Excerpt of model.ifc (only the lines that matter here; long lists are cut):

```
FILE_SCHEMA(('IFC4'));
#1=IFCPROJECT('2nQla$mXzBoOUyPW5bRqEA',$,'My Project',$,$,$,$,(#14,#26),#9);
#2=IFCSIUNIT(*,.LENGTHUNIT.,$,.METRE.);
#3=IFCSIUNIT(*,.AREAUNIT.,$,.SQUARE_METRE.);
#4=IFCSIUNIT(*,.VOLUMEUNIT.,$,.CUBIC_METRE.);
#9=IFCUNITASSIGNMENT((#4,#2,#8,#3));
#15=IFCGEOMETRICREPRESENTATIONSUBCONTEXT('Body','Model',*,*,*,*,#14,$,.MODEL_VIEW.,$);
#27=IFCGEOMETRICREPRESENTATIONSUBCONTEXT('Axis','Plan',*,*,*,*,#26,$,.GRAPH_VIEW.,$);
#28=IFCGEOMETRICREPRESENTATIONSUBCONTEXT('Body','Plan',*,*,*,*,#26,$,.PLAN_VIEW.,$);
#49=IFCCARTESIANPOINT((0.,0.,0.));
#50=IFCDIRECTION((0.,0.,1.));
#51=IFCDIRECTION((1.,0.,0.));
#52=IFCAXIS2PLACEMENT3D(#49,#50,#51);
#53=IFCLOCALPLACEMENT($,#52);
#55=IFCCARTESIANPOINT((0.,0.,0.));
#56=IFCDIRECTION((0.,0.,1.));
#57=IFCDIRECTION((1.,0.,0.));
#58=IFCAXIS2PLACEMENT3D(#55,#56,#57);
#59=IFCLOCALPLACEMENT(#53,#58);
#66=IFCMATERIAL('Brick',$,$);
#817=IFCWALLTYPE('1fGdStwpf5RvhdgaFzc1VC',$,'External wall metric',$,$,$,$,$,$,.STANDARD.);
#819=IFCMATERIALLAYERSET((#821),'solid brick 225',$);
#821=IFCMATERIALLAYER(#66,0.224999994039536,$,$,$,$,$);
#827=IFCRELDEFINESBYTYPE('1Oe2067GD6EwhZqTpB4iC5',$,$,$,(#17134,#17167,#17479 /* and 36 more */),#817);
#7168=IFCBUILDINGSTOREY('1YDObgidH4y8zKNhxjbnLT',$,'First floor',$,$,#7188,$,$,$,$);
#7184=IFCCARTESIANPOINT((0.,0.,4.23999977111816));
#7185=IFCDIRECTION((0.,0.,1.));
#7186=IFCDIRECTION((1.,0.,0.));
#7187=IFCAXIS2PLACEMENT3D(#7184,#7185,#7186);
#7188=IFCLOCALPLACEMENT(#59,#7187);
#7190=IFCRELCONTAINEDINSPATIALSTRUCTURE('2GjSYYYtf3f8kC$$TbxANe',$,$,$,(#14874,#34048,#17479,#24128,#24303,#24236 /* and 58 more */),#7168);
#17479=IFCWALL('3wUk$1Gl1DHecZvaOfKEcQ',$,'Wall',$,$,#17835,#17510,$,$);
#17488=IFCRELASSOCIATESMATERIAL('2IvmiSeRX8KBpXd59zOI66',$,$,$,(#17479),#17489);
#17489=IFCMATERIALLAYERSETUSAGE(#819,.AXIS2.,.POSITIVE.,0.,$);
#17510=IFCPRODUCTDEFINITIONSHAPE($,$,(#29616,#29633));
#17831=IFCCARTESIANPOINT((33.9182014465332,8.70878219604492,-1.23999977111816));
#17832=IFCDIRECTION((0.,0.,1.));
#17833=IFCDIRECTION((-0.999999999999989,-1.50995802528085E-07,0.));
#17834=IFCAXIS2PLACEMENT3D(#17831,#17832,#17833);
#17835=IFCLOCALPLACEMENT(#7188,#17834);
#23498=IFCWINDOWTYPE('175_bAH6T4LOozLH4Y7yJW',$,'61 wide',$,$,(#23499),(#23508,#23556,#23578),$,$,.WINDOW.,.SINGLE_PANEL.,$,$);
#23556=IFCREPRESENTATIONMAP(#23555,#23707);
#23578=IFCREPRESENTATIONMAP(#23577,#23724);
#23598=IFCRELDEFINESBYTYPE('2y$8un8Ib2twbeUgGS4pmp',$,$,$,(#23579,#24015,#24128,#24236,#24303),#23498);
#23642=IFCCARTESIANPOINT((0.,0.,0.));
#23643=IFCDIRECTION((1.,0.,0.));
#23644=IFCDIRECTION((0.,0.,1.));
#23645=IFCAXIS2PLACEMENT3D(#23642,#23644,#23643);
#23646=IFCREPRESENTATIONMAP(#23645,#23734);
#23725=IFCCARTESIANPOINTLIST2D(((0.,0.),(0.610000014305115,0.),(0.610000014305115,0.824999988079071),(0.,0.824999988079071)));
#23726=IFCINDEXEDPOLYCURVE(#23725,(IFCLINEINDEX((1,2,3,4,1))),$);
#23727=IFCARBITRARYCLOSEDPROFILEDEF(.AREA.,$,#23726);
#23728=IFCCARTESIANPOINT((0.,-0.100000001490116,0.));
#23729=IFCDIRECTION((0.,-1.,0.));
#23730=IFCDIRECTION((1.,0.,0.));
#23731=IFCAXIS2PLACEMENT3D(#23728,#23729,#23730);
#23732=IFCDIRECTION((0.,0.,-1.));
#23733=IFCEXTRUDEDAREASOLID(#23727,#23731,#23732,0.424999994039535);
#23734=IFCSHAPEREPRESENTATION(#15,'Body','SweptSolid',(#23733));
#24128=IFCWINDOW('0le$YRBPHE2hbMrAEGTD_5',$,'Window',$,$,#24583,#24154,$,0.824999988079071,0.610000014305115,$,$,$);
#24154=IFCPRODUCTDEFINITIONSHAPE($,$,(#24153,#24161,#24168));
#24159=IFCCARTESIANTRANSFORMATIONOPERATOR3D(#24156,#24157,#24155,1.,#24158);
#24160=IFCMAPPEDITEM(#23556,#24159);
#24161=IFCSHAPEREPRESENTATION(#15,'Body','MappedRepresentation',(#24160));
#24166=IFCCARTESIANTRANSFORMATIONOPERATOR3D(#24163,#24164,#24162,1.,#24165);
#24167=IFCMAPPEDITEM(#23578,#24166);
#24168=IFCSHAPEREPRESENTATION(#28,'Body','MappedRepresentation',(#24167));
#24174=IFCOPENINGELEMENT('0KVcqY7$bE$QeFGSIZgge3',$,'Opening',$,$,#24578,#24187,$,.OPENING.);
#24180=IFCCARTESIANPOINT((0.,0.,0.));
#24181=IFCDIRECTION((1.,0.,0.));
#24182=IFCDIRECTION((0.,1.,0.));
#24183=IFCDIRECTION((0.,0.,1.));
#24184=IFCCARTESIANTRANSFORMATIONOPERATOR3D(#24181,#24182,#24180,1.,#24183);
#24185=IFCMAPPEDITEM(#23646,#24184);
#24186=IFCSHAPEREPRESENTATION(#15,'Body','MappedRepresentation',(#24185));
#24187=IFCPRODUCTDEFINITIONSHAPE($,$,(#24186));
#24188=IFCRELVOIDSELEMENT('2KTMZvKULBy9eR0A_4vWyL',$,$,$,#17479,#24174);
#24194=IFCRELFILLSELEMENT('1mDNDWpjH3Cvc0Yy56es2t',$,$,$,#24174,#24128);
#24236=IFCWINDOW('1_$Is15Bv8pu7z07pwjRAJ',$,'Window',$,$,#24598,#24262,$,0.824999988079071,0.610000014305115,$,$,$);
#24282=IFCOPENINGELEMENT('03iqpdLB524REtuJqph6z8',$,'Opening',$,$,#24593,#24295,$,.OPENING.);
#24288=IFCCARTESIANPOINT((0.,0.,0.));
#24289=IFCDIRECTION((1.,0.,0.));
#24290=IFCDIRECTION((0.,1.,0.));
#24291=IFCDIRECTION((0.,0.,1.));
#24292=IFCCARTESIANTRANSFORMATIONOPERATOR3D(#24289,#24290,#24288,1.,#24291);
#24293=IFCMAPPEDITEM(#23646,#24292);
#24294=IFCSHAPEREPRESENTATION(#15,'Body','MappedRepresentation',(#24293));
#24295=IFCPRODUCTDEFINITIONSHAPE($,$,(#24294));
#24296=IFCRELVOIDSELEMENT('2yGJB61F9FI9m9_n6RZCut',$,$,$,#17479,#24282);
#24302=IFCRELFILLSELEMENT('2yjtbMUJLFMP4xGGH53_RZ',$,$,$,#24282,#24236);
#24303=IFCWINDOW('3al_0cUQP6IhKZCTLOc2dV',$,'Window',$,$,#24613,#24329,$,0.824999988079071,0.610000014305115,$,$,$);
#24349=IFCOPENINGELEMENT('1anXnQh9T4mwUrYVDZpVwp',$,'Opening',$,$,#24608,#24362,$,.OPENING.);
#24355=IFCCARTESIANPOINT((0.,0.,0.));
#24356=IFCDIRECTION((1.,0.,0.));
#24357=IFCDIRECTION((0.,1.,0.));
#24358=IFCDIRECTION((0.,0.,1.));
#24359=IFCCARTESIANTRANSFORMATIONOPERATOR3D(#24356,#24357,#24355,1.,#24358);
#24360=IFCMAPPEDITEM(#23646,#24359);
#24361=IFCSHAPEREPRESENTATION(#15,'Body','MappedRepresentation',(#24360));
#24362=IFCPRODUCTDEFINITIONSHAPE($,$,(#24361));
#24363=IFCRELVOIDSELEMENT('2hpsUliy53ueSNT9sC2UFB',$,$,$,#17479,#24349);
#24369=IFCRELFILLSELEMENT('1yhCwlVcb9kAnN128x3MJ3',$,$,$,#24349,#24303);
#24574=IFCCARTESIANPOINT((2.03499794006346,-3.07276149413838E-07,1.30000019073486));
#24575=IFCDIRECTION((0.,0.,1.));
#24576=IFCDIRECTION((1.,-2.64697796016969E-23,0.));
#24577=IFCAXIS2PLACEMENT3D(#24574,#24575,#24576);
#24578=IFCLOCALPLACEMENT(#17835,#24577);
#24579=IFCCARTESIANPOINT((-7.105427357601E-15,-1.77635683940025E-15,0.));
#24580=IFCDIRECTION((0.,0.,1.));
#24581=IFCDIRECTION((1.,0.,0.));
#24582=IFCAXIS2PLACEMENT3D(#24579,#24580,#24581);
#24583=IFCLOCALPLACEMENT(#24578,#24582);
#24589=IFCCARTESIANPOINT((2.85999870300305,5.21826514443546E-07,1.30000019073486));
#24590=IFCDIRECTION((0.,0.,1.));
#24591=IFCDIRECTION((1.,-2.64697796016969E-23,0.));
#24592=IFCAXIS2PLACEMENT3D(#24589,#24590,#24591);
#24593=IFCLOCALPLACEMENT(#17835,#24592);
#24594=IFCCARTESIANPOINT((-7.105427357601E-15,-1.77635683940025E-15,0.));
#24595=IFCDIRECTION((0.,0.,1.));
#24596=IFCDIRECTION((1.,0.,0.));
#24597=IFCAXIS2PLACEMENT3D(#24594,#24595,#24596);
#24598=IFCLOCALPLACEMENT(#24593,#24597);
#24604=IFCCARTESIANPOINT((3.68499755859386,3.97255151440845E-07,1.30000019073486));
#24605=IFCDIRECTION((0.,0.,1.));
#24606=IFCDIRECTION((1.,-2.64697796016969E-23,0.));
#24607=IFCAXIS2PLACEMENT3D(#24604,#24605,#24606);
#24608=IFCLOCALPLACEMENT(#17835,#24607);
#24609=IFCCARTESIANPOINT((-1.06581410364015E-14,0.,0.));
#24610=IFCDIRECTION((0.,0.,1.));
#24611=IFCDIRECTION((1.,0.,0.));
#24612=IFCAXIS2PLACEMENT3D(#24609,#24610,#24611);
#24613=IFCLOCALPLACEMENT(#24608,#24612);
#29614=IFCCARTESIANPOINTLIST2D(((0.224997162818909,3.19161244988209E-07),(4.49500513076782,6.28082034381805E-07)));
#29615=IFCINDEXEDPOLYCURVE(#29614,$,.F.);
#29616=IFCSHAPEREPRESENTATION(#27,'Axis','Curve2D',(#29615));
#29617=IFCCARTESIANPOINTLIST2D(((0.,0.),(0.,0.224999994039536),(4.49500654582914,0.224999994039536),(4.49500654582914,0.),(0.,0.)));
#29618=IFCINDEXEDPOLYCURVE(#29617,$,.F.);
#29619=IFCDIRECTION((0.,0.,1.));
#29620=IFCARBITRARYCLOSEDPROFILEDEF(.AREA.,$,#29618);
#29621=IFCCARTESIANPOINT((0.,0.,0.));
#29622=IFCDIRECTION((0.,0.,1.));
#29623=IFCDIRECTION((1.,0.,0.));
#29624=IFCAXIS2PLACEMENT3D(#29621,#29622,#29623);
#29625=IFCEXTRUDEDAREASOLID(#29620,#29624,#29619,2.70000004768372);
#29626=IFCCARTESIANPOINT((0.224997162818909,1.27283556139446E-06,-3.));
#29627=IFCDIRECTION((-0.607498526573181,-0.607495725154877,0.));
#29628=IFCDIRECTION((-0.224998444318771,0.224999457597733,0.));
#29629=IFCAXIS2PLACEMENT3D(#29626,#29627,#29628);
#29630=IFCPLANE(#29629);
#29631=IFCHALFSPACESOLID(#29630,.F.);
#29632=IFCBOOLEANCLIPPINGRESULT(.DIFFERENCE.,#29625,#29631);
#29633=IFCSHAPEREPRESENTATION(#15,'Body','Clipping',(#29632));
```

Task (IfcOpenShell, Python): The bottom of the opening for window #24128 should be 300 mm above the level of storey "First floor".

```python
import numpy as np
import ifcopenshell
import ifcopenshell.api.geometry
import ifcopenshell.geom
import ifcopenshell.util.element
import ifcopenshell.util.placement
import ifcopenshell.util.shape
import ifcopenshell.util.unit

model = ifcopenshell.open("model.ifc")
unit_scale = ifcopenshell.util.unit.calculate_unit_scale(model)

window = model.by_guid("0le$YRBPHE2hbMrAEGTD_5")
opening = window.FillsVoids[0].RelatingOpeningElement
storey = ifcopenshell.util.element.get_container(window, ifc_class="IfcBuildingStorey")
level = ifcopenshell.util.placement.get_local_placement(storey.ObjectPlacement)[2, 3]

# The opening's origin need not be at the sill, so measure its lowest point.
shape = ifcopenshell.geom.create_shape(ifcopenshell.geom.settings(), opening)
bottom = ifcopenshell.util.shape.get_shape_bottom_elevation(shape, shape.geometry) / unit_scale
dz = level + 0.3 / unit_scale - bottom

shift = np.array([0.0, 0.0, dz])
# The window is placed relative to its opening, so it follows when the opening moves.
matrix = ifcopenshell.util.placement.get_local_placement(opening.ObjectPlacement)
matrix[:3, 3] += shift
ifcopenshell.api.geometry.edit_object_placement(
    model, product=opening, matrix=matrix, is_si=False, should_transform_children=True
)

print(f"moved by {dz * unit_scale:+.3f} m")

model.write("model_updated.ifc")
```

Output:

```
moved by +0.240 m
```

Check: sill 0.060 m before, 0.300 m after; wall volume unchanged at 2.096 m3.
